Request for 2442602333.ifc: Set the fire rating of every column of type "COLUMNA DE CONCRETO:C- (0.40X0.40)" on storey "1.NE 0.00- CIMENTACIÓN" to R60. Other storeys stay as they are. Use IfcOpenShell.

First a look at what the model holds.

```python
import ifcopenshell
import ifcopenshell.util.element

model = ifcopenshell.open("2442602333.ifc")
print(model.schema)
storey = next(s for s in model.by_type("IfcBuildingStorey") if s.Name == "1.NE 0.00- CIMENTACIÓN")
columns = [e for e in ifcopenshell.util.element.get_decomposition(storey) if e.is_a("IfcColumn")]
seen = {}
for e in columns:
    element_type = ifcopenshell.util.element.get_type(e)
    key = (element_type.Name if element_type != e and element_type else None, ifcopenshell.util.element.get_pset(e, "Pset_ColumnCommon", "FireRating"))
    seen[key] = seen.get(key, 0) + 1
for (name, value), count in sorted(seen.items(), key=str):
    print(count, "x", name, "|", value)
```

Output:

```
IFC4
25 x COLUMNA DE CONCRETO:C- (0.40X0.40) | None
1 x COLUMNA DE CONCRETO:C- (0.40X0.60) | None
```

```python
import ifcopenshell
import ifcopenshell.api.pset
import ifcopenshell.util.element

model = ifcopenshell.open("2442602333.ifc")

storey = next(s for s in model.by_type("IfcBuildingStorey") if s.Name == "1.NE 0.00- CIMENTACIÓN")
columns = [e for e in ifcopenshell.util.element.get_decomposition(storey) if e.is_a("IfcColumn")]

count = 0
for e in columns:
    element_type = ifcopenshell.util.element.get_type(e)
    if element_type in (None, e) or element_type.Name != "COLUMNA DE CONCRETO:C- (0.40X0.40)":
        continue
    # add_pset returns the element's existing set when there is one.
    pset = ifcopenshell.api.pset.add_pset(model, product=e, name="Pset_ColumnCommon")
    ifcopenshell.api.pset.edit_pset(model, pset=pset, properties={"FireRating": "R60"})
    count += 1

print(count, "columns updated")

model.write("2442602333-out.ifc")
```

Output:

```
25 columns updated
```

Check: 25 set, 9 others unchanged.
